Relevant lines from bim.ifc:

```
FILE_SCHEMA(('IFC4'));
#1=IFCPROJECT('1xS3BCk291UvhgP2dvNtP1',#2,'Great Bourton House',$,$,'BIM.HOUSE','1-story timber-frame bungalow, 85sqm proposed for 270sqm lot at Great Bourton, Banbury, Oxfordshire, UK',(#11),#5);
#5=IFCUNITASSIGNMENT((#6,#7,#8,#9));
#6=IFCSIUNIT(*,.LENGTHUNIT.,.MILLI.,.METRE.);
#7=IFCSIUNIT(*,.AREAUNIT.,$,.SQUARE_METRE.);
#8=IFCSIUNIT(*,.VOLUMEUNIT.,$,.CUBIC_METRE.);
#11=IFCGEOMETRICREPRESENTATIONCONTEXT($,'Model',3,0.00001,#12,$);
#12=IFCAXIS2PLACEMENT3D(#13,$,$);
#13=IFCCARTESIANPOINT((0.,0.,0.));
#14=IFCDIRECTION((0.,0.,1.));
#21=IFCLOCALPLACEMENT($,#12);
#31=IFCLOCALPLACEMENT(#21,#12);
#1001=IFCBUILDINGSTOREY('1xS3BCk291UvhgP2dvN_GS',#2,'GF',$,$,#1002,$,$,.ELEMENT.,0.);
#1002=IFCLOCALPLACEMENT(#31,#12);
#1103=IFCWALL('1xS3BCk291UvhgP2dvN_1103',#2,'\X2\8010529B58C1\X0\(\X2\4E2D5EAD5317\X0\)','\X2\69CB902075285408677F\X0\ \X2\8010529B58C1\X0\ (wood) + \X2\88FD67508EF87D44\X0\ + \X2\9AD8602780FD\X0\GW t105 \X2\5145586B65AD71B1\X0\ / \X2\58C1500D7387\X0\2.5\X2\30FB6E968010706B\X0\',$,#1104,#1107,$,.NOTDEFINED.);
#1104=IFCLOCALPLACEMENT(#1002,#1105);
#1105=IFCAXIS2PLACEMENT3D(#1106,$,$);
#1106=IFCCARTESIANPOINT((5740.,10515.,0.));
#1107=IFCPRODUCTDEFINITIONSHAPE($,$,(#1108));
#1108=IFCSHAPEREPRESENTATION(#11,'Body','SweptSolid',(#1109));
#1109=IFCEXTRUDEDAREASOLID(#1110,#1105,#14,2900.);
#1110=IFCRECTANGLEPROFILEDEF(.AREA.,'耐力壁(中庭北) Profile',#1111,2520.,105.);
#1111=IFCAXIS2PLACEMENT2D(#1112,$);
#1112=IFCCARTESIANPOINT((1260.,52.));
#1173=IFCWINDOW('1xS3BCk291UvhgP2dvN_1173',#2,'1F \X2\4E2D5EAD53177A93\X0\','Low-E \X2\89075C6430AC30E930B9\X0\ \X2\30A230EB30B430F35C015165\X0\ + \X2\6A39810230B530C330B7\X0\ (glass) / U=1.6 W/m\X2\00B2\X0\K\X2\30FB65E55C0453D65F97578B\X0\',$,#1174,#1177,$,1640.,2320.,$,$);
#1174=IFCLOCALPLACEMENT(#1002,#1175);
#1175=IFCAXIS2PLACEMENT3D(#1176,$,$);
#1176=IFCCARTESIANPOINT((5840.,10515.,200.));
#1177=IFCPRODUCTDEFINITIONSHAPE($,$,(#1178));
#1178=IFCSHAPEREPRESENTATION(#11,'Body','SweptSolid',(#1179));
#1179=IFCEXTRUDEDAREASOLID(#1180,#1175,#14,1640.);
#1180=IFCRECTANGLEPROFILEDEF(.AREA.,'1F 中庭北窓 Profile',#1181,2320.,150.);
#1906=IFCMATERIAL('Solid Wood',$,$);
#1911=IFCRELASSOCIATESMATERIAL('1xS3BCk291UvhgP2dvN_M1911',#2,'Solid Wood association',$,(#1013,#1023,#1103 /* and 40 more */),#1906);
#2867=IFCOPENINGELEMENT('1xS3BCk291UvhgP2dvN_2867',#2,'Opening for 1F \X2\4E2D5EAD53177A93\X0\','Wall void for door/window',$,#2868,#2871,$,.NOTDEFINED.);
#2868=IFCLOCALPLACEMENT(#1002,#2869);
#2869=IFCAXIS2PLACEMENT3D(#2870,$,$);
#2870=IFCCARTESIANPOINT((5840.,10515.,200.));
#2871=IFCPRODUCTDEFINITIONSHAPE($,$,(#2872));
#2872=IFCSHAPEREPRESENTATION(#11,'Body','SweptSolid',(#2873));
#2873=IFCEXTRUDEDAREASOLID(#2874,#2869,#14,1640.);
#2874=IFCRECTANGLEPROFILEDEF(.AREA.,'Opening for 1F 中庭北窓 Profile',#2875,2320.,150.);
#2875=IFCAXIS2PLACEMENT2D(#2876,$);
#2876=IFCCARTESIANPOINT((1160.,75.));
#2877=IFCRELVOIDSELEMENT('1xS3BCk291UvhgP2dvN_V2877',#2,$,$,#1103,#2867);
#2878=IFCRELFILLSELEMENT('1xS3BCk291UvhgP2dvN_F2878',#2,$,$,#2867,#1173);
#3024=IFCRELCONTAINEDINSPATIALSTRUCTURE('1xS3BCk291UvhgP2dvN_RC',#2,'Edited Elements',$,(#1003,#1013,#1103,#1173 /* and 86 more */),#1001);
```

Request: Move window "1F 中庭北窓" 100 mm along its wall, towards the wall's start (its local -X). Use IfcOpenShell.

```python
import ifcopenshell
import ifcopenshell.api.geometry
import ifcopenshell.util.placement
import ifcopenshell.util.unit

model = ifcopenshell.open("bim.ifc")
unit_scale = ifcopenshell.util.unit.calculate_unit_scale(model)

window = model.by_guid("1xS3BCk291UvhgP2dvN_1173")
opening = window.FillsVoids[0].RelatingOpeningElement
wall = opening.VoidsElements[0].RelatingBuildingElement

wall_matrix = ifcopenshell.util.placement.get_local_placement(wall.ObjectPlacement)
shift = wall_matrix[:3, 0] * -0.1 / unit_scale
before = ifcopenshell.util.placement.get_local_placement(window.ObjectPlacement)[:3, 3].copy()

# The window is not placed relative to its opening, so move both.
for product in (opening, window):
    matrix = ifcopenshell.util.placement.get_local_placement(product.ObjectPlacement)
    matrix[:3, 3] += shift
    ifcopenshell.api.geometry.edit_object_placement(model, product=product, matrix=matrix, is_si=False)

after = ifcopenshell.util.placement.get_local_placement(window.ObjectPlacement)[:3, 3]
print("window moved by", (after - before).round(3) + 0.0)

model.write("bim_rev.ifc")
```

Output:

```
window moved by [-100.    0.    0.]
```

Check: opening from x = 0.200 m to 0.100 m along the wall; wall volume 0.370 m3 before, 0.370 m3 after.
